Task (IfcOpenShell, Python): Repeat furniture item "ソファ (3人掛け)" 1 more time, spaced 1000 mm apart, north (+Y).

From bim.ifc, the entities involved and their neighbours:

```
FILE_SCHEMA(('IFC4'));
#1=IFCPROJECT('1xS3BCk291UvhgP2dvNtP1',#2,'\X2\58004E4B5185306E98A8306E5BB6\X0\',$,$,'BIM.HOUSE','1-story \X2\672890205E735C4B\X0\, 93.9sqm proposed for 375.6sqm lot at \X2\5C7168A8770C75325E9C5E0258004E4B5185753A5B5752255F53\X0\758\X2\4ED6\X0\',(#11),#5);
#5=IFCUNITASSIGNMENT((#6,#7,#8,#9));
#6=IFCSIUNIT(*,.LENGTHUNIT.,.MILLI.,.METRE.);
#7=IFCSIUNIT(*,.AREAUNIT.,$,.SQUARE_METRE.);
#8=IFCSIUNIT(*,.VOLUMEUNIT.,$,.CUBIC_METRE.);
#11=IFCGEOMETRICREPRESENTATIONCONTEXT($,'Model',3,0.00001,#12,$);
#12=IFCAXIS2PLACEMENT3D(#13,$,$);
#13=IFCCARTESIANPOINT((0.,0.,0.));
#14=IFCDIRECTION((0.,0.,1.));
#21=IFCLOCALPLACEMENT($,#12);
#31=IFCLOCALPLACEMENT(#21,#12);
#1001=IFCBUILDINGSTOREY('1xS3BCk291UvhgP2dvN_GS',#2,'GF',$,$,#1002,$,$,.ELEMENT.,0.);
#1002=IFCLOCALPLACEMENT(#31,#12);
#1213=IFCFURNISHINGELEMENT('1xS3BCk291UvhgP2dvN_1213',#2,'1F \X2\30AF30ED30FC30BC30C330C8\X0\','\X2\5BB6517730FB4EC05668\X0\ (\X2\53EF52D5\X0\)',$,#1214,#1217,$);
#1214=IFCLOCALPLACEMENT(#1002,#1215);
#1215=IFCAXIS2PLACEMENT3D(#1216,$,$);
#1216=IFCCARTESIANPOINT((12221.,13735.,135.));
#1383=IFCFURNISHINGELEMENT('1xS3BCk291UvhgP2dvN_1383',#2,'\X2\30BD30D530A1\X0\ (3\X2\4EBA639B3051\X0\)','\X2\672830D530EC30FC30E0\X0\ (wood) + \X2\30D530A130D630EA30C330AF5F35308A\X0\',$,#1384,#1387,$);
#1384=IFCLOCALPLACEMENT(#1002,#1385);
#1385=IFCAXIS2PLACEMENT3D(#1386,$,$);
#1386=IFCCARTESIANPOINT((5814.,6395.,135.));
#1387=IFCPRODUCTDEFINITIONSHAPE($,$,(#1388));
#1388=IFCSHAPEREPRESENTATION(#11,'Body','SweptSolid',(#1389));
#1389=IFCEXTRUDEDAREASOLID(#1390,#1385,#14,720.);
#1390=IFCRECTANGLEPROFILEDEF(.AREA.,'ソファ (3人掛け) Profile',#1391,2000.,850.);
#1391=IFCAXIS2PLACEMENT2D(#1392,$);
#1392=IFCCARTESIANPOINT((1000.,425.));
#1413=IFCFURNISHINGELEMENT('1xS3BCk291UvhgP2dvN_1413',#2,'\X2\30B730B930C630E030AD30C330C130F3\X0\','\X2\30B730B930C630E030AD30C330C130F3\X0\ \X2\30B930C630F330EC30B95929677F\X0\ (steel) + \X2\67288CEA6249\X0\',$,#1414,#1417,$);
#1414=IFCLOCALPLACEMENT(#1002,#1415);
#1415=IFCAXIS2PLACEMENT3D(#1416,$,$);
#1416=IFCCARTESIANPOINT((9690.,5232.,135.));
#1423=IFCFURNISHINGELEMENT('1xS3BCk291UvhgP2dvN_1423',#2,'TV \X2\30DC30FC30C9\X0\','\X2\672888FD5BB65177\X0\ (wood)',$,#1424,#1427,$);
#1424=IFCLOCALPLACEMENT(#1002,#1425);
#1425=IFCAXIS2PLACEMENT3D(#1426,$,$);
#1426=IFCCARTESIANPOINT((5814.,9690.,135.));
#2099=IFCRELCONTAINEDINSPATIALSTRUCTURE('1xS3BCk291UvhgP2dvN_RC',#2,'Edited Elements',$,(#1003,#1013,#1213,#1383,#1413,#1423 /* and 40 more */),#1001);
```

```python
import numpy as np
import ifcopenshell
import ifcopenshell.api.geometry
import ifcopenshell.api.root
import ifcopenshell.util.element
import ifcopenshell.util.placement
import ifcopenshell.util.unit

model = ifcopenshell.open("bim.ifc")
unit_scale = ifcopenshell.util.unit.calculate_unit_scale(model)


def reuse_history(source, copy):
    """copy_class also copies each property set's owner history, people and application; keep the originals."""
    for rel in copy.IsDefinedBy:
        if rel.is_a("IfcRelDefinesByProperties") and (history := rel.RelatingPropertyDefinition.OwnerHistory):
            rel.RelatingPropertyDefinition.OwnerHistory = source.OwnerHistory
            ifcopenshell.util.element.remove_deep2(model, history)


source = model.by_guid("1xS3BCk291UvhgP2dvN_1383")
base = ifcopenshell.util.placement.get_local_placement(source.ObjectPlacement)
step = np.array([0.0, 1.0, 0.0]) * 1 / unit_scale

for i in range(1, 2):
    copy = ifcopenshell.api.root.copy_class(model, product=source)
    copy.Representation = ifcopenshell.util.element.copy_deep(
        model, source.Representation, exclude=["IfcGeometricRepresentationContext", "IfcRepresentationMap"]
    )
    reuse_history(source, copy)
    matrix = base.copy()
    matrix[:3, 3] += i * step
    print("added at", matrix[:3, 3].round(3) + 0.0)
    ifcopenshell.api.geometry.edit_object_placement(model, product=copy, matrix=matrix, is_si=False)

model.write("bim_edited.ifc")
```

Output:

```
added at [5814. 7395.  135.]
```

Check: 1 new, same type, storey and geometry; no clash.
